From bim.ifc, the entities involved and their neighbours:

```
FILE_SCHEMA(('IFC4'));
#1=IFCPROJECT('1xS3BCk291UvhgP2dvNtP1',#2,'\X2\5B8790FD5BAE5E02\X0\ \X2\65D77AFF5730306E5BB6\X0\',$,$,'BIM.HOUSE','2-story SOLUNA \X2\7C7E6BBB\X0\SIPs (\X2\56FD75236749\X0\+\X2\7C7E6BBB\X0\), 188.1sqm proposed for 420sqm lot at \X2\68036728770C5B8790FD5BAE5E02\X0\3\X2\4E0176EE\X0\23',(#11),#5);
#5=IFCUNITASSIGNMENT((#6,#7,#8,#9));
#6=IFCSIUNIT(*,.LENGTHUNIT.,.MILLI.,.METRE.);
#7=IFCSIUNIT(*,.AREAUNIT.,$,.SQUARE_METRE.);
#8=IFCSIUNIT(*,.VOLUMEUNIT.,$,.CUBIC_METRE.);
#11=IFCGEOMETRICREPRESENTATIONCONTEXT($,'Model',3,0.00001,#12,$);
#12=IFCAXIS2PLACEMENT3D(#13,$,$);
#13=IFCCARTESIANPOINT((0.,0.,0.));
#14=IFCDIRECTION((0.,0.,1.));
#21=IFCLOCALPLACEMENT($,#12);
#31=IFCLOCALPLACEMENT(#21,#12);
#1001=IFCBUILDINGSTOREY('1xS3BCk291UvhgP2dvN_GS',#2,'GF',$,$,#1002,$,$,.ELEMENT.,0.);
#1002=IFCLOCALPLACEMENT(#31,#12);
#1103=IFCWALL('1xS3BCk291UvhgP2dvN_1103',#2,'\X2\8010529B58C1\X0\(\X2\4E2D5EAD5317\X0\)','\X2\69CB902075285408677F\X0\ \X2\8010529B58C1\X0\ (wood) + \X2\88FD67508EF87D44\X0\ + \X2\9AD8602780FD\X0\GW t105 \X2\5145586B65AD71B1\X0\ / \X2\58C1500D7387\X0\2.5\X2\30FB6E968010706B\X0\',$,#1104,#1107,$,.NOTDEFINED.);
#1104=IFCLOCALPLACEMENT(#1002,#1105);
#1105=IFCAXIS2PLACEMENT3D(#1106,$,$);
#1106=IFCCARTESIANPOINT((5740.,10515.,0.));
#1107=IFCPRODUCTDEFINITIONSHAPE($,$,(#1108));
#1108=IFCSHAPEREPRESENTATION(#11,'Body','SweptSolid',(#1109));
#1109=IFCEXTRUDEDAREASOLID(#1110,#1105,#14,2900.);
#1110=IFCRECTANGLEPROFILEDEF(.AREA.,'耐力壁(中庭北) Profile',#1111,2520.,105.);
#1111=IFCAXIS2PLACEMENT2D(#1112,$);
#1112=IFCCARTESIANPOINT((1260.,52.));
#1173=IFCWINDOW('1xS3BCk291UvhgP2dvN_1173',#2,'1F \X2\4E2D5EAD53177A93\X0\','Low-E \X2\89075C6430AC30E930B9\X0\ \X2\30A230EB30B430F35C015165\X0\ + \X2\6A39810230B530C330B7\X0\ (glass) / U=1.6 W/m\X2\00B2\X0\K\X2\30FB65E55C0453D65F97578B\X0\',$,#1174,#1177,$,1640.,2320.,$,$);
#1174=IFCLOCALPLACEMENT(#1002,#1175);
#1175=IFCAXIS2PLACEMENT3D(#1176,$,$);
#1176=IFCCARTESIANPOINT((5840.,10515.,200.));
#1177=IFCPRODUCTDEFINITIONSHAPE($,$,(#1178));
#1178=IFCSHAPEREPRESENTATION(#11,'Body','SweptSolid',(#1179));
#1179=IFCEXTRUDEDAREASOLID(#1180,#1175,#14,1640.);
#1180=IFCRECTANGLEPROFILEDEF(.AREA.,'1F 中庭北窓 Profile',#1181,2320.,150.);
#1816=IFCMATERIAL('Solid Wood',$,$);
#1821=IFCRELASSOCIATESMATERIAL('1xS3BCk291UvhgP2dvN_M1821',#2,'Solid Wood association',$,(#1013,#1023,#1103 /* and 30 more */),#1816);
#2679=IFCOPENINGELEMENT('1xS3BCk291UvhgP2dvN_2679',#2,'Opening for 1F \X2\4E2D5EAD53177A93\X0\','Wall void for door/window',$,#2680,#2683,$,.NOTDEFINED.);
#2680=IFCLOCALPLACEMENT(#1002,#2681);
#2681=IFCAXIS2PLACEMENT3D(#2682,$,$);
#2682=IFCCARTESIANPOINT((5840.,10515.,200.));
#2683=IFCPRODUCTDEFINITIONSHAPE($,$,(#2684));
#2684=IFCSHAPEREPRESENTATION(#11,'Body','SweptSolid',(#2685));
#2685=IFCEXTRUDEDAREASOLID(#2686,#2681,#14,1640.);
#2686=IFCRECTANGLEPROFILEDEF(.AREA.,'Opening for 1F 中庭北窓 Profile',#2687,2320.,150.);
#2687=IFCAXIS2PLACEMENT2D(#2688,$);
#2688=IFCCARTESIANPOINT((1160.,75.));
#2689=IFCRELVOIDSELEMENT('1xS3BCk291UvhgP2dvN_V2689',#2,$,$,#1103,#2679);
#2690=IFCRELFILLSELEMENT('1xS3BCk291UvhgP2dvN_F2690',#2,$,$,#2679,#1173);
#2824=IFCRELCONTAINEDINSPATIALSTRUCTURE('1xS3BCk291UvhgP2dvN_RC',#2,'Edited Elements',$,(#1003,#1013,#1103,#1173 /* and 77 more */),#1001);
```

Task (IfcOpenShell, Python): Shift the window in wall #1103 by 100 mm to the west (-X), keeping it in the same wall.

```python
import ifcopenshell
import ifcopenshell.api.geometry
import ifcopenshell.util.placement

model = ifcopenshell.open("bim.ifc")

window = model.by_id(1173)
opening = window.FillsVoids[0].RelatingOpeningElement
wall = opening.VoidsElements[0].RelatingBuildingElement

wall_matrix = ifcopenshell.util.placement.get_local_placement(wall.ObjectPlacement)
shift = wall_matrix[:3, 0] * -100.0
before = ifcopenshell.util.placement.get_local_placement(window.ObjectPlacement)[:3, 3].copy()

# The window is not placed relative to its opening, so move both.
for product in (opening, window):
    matrix = ifcopenshell.util.placement.get_local_placement(product.ObjectPlacement)
    matrix[:3, 3] += shift
    ifcopenshell.api.geometry.edit_object_placement(model, product=product, matrix=matrix, is_si=False)

after = ifcopenshell.util.placement.get_local_placement(window.ObjectPlacement)[:3, 3]
print("window moved by", (after - before).round(3) + 0.0)

model.write("bim_updated.ifc")
```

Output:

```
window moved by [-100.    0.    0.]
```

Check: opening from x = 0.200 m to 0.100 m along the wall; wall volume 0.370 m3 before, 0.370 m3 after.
